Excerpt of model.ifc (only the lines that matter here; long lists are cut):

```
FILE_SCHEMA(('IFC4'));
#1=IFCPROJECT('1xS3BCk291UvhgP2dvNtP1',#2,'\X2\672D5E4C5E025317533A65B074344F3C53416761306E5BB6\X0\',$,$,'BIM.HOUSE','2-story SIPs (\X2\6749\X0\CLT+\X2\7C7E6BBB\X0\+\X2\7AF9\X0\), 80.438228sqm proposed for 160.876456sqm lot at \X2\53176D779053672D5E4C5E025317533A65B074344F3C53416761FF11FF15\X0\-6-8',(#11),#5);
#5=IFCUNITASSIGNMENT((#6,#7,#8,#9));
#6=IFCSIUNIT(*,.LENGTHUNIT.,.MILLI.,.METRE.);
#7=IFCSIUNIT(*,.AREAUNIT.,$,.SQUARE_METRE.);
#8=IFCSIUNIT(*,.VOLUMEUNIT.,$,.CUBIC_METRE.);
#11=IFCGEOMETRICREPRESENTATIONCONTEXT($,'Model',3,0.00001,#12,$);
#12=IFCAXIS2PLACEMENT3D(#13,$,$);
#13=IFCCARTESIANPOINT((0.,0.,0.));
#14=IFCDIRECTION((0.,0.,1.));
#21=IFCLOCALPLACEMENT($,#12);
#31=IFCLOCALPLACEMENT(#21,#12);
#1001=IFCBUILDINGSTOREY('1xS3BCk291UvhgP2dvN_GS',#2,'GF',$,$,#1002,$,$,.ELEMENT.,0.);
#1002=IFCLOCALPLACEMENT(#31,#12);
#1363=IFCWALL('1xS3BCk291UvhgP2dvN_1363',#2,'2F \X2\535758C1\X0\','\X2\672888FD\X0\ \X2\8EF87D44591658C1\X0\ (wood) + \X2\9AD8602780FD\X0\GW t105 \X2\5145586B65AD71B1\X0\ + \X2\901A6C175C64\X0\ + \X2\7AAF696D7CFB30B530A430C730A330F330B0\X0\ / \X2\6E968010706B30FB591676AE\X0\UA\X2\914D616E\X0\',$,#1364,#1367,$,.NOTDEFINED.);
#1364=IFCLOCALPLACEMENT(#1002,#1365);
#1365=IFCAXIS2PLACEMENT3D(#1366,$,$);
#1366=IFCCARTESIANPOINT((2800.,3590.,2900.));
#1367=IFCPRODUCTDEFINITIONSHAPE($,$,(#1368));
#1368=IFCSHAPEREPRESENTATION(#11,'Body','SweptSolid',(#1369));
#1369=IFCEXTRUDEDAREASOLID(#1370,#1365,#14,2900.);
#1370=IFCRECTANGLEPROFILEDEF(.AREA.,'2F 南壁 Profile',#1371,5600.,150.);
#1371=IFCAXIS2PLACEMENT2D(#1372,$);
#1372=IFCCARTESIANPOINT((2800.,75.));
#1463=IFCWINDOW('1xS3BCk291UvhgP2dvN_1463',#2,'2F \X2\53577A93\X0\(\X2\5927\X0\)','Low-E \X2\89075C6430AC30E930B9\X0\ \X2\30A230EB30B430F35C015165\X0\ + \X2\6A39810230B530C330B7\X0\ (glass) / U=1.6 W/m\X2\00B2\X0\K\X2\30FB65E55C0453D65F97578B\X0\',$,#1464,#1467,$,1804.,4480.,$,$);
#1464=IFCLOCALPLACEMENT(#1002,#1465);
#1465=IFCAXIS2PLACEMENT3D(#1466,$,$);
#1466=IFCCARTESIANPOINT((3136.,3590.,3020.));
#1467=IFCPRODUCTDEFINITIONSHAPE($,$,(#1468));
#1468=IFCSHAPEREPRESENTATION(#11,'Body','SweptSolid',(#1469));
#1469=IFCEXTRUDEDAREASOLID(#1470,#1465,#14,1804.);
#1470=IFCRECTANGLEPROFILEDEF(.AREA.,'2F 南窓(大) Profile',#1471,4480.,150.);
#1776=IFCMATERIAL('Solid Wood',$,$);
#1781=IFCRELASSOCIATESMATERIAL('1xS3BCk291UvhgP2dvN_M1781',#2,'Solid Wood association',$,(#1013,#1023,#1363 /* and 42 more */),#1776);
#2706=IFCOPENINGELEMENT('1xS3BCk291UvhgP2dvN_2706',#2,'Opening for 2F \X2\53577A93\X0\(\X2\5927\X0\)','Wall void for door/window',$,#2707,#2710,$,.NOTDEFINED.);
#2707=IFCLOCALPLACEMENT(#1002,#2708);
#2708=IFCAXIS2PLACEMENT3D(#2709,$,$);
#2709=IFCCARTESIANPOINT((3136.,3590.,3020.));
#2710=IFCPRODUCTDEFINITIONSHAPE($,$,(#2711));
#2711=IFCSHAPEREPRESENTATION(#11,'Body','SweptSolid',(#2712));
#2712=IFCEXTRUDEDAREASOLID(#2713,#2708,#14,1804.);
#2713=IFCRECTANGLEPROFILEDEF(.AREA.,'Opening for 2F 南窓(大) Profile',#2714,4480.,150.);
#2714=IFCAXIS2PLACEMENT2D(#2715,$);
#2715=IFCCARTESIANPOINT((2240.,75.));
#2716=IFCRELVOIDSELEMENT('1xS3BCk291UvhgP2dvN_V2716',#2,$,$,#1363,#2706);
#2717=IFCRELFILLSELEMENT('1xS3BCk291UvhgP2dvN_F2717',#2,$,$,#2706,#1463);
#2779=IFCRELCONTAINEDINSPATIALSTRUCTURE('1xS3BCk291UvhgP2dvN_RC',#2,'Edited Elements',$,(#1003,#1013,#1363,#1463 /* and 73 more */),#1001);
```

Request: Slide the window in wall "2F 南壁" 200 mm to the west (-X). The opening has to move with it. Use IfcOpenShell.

```python
import ifcopenshell
import ifcopenshell.api.geometry
import ifcopenshell.util.placement

model = ifcopenshell.open("model.ifc")

window = model.by_guid("1xS3BCk291UvhgP2dvN_1463")
opening = window.FillsVoids[0].RelatingOpeningElement
wall = opening.VoidsElements[0].RelatingBuildingElement

wall_matrix = ifcopenshell.util.placement.get_local_placement(wall.ObjectPlacement)
shift = wall_matrix[:3, 0] * -200.0
before = ifcopenshell.util.placement.get_local_placement(window.ObjectPlacement)[:3, 3].copy()

# The window is not placed relative to its opening, so move both.
for product in (opening, window):
    matrix = ifcopenshell.util.placement.get_local_placement(product.ObjectPlacement)
    matrix[:3, 3] += shift
    ifcopenshell.api.geometry.edit_object_placement(model, product=product, matrix=matrix, is_si=False)

after = ifcopenshell.util.placement.get_local_placement(window.ObjectPlacement)[:3, 3]
print("window moved by", (after - before).round(3) + 0.0)

model.write("model_edited.ifc")
```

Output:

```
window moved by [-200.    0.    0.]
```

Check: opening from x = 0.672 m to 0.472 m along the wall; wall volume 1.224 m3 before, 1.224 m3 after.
